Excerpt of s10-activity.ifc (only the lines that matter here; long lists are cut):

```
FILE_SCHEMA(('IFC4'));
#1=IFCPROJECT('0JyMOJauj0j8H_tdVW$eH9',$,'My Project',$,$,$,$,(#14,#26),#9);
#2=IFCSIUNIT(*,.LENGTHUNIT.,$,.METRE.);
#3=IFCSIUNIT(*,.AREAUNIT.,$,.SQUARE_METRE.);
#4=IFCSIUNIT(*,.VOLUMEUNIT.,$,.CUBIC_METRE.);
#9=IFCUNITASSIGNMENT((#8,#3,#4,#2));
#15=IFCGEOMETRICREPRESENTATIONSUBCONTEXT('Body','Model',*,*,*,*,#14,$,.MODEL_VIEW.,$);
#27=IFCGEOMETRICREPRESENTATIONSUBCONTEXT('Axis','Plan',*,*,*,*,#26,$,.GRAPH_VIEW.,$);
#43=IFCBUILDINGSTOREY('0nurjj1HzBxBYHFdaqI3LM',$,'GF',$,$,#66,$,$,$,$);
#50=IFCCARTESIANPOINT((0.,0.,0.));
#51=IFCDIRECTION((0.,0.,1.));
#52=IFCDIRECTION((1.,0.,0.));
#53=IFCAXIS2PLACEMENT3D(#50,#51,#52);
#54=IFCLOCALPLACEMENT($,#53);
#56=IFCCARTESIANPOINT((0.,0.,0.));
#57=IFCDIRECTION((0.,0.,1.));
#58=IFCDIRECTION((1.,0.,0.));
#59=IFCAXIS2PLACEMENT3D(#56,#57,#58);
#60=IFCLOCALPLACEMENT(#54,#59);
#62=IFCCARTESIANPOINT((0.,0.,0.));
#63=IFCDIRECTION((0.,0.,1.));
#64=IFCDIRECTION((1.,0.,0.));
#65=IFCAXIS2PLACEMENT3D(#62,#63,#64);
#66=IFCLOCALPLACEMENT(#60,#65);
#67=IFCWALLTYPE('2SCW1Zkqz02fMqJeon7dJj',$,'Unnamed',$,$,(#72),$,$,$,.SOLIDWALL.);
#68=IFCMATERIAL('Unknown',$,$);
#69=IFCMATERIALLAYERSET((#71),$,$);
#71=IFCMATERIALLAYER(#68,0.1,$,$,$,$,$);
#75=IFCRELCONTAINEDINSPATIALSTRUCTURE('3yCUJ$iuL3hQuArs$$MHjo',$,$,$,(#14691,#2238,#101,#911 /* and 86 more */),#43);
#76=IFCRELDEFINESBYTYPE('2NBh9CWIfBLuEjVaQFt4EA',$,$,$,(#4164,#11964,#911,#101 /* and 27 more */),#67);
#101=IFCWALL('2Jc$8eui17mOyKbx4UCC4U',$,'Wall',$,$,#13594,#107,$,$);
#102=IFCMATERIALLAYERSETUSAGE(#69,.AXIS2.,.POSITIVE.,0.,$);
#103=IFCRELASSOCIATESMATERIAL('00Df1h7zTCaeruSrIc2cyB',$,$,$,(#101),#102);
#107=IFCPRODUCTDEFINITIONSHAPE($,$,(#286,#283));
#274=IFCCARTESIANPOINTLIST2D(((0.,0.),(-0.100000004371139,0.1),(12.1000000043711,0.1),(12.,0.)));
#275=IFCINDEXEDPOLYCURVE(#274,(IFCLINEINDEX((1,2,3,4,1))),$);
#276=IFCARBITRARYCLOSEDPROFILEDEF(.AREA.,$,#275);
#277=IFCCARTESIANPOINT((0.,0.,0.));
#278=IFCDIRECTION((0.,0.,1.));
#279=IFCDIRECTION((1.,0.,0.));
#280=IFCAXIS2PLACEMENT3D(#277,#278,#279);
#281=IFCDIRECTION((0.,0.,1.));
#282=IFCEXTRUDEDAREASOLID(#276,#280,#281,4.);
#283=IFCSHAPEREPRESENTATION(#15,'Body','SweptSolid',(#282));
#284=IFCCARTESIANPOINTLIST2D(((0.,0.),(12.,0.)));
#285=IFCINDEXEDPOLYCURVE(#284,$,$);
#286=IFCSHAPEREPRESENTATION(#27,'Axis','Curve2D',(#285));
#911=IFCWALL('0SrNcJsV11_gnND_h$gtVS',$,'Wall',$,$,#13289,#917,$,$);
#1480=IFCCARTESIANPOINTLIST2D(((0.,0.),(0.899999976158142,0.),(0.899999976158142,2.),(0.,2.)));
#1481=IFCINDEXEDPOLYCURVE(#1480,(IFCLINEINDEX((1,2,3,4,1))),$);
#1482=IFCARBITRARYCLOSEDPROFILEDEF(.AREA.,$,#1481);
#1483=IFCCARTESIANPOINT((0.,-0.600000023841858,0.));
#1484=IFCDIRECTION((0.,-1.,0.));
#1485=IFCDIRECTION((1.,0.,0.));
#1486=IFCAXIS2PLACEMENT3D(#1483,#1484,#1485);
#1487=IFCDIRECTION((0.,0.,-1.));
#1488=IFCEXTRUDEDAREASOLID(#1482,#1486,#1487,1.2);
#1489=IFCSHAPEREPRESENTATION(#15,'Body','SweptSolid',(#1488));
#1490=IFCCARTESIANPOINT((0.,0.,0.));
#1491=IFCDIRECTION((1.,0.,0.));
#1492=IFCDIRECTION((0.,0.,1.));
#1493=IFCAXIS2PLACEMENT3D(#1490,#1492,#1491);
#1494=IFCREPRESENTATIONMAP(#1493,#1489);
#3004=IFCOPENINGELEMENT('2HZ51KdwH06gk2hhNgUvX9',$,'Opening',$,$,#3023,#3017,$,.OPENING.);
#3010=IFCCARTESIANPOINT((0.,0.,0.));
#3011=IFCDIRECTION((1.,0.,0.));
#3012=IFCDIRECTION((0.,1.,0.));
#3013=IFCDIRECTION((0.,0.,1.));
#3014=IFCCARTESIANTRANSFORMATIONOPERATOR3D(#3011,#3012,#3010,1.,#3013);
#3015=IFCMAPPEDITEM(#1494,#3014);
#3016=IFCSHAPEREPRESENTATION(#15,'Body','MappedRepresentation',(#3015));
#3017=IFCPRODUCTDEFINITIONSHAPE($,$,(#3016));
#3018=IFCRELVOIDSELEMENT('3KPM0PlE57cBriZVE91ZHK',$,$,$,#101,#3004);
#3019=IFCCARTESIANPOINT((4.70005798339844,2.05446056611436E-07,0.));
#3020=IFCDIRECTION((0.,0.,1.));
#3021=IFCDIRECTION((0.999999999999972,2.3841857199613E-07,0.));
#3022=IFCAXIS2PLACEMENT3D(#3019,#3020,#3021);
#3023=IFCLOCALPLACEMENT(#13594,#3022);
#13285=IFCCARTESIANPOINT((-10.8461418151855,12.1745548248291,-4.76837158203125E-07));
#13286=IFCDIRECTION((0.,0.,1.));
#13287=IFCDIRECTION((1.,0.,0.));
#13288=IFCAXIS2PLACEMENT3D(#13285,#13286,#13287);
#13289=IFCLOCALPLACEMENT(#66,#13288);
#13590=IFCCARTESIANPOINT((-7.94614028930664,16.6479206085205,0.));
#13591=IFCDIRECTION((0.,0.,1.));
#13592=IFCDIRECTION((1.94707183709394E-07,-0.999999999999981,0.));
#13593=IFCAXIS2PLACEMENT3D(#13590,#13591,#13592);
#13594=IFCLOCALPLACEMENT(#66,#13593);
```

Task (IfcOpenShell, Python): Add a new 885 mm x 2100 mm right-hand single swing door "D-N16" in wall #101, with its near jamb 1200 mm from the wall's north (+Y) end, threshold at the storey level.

```python
import numpy as np
import ifcopenshell
import ifcopenshell.api.feature
import ifcopenshell.api.geometry
import ifcopenshell.api.root
import ifcopenshell.api.spatial
import ifcopenshell.geom
import ifcopenshell.util.element
import ifcopenshell.util.placement
import ifcopenshell.util.representation
import ifcopenshell.util.shape
import ifcopenshell.util.unit

model = ifcopenshell.open("s10-activity.ifc")
unit_scale = ifcopenshell.util.unit.calculate_unit_scale(model)
settings = ifcopenshell.geom.settings()


def volume(element):
    """Net volume in cubic metres, openings subtracted."""
    shape = ifcopenshell.geom.create_shape(settings, element)
    return ifcopenshell.util.shape.get_volume(shape.geometry)


wall = model.by_guid("2Jc$8eui17mOyKbx4UCC4U")
storey = ifcopenshell.util.element.get_container(wall, ifc_class="IfcBuildingStorey")
context = ifcopenshell.util.representation.get_context(model, "Model", "Body", "MODEL_VIEW")
before = volume(wall)

width, height, from_end, sill = 0.885, 2.1, 1.2, 0.0  # metres

# The wall runs along its own X axis, and the end named is its -X end.
wall_shape = ifcopenshell.geom.create_shape(settings, wall)
x, y, z = ifcopenshell.util.shape.get_vertices(wall_shape.geometry).T
start = x.min() + from_end
face, thickness = float(y.min()), float(y.max() - y.min())
wall_matrix = ifcopenshell.util.placement.get_local_placement(wall.ObjectPlacement)
level = ifcopenshell.util.placement.get_local_placement(storey.ObjectPlacement)[2, 3]


def in_wall(x, y):
    """Placement at x, y metres in the wall's axes, at sill height."""
    matrix = wall_matrix.copy()
    matrix[:, 3] = wall_matrix @ np.array([x / unit_scale, y / unit_scale, 0.0, 1.0])
    matrix[2, 3] = level + sill / unit_scale
    return matrix


# Opening: a box that overshoots both wall faces by 50 mm.
opening = ifcopenshell.api.root.create_entity(model, ifc_class="IfcOpeningElement", predefined_type="OPENING")
box = ifcopenshell.api.geometry.add_wall_representation(
    model, context=context, length=width, height=height, thickness=thickness + 0.1
)
ifcopenshell.api.geometry.assign_representation(model, product=opening, representation=box)
ifcopenshell.api.geometry.edit_object_placement(model, product=opening, matrix=in_wall(start, face - 0.05), is_si=False)
ifcopenshell.api.feature.add_feature(model, feature=opening, element=wall)

door = ifcopenshell.api.root.create_entity(model, ifc_class="IfcDoor", name="D-N16", predefined_type="DOOR")
door.OverallWidth, door.OverallHeight = width / unit_scale, height / unit_scale
door.OperationType = "SINGLE_SWING_RIGHT"
body = ifcopenshell.api.geometry.add_door_representation(
    model,
    context=context,
    overall_width=door.OverallWidth,
    overall_height=door.OverallHeight,
    operation_type="SINGLE_SWING_RIGHT",
    lining_properties={"LiningDepth": thickness / unit_scale, "ThresholdDepth": thickness / unit_scale},
)
ifcopenshell.api.geometry.assign_representation(model, product=door, representation=body)
ifcopenshell.api.spatial.assign_container(model, products=[door], relating_structure=storey)
ifcopenshell.api.feature.add_filling(model, opening=opening, element=door)

# The lining spans the wall, so the door starts at the wall face.
ifcopenshell.api.geometry.edit_object_placement(model, product=door, matrix=in_wall(start, face), is_si=False)

after = volume(wall)

print(f"wall volume {before:.3f} -> {after:.3f} m3")

model.write("s10-activity_v2.ifc")
```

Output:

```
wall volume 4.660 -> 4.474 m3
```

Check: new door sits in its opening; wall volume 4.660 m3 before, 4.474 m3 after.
